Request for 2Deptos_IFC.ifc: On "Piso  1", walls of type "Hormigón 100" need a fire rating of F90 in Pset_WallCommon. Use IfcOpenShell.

First a look at what the model holds.

```python
import ifcopenshell
import ifcopenshell.util.element

model = ifcopenshell.open("2Deptos_IFC.ifc")
print(model.schema)
storey = next(s for s in model.by_type("IfcBuildingStorey") if s.Name == "Piso  1")
walls = [e for e in ifcopenshell.util.element.get_decomposition(storey) if e.is_a("IfcWall")]
seen = {}
for e in walls:
    element_type = ifcopenshell.util.element.get_type(e)
    key = (element_type.Name if element_type != e and element_type else None, ifcopenshell.util.element.get_pset(e, "Pset_WallCommon", "FireRating"))
    seen[key] = seen.get(key, 0) + 1
for (name, value), count in sorted(seen.items(), key=str):
    print(count, "x", name, "|", value)
```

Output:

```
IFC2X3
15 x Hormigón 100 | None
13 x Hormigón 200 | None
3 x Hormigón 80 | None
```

```python
import ifcopenshell
import ifcopenshell.api.pset
import ifcopenshell.util.element

model = ifcopenshell.open("2Deptos_IFC.ifc")

storey = next(s for s in model.by_type("IfcBuildingStorey") if s.Name == "Piso  1")
walls = [e for e in ifcopenshell.util.element.get_decomposition(storey) if e.is_a("IfcWall")]

count = 0
for e in walls:
    element_type = ifcopenshell.util.element.get_type(e)
    if element_type in (None, e) or element_type.Name != "Hormigón 100":
        continue
    # add_pset returns the element's existing set when there is one.
    pset = ifcopenshell.api.pset.add_pset(model, product=e, name="Pset_WallCommon")
    ifcopenshell.api.pset.edit_pset(model, pset=pset, properties={"FireRating": "F90"})
    count += 1

print(count, "walls updated")

model.write("2Deptos_IFC_updated.ifc")
```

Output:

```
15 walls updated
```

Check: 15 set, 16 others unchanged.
